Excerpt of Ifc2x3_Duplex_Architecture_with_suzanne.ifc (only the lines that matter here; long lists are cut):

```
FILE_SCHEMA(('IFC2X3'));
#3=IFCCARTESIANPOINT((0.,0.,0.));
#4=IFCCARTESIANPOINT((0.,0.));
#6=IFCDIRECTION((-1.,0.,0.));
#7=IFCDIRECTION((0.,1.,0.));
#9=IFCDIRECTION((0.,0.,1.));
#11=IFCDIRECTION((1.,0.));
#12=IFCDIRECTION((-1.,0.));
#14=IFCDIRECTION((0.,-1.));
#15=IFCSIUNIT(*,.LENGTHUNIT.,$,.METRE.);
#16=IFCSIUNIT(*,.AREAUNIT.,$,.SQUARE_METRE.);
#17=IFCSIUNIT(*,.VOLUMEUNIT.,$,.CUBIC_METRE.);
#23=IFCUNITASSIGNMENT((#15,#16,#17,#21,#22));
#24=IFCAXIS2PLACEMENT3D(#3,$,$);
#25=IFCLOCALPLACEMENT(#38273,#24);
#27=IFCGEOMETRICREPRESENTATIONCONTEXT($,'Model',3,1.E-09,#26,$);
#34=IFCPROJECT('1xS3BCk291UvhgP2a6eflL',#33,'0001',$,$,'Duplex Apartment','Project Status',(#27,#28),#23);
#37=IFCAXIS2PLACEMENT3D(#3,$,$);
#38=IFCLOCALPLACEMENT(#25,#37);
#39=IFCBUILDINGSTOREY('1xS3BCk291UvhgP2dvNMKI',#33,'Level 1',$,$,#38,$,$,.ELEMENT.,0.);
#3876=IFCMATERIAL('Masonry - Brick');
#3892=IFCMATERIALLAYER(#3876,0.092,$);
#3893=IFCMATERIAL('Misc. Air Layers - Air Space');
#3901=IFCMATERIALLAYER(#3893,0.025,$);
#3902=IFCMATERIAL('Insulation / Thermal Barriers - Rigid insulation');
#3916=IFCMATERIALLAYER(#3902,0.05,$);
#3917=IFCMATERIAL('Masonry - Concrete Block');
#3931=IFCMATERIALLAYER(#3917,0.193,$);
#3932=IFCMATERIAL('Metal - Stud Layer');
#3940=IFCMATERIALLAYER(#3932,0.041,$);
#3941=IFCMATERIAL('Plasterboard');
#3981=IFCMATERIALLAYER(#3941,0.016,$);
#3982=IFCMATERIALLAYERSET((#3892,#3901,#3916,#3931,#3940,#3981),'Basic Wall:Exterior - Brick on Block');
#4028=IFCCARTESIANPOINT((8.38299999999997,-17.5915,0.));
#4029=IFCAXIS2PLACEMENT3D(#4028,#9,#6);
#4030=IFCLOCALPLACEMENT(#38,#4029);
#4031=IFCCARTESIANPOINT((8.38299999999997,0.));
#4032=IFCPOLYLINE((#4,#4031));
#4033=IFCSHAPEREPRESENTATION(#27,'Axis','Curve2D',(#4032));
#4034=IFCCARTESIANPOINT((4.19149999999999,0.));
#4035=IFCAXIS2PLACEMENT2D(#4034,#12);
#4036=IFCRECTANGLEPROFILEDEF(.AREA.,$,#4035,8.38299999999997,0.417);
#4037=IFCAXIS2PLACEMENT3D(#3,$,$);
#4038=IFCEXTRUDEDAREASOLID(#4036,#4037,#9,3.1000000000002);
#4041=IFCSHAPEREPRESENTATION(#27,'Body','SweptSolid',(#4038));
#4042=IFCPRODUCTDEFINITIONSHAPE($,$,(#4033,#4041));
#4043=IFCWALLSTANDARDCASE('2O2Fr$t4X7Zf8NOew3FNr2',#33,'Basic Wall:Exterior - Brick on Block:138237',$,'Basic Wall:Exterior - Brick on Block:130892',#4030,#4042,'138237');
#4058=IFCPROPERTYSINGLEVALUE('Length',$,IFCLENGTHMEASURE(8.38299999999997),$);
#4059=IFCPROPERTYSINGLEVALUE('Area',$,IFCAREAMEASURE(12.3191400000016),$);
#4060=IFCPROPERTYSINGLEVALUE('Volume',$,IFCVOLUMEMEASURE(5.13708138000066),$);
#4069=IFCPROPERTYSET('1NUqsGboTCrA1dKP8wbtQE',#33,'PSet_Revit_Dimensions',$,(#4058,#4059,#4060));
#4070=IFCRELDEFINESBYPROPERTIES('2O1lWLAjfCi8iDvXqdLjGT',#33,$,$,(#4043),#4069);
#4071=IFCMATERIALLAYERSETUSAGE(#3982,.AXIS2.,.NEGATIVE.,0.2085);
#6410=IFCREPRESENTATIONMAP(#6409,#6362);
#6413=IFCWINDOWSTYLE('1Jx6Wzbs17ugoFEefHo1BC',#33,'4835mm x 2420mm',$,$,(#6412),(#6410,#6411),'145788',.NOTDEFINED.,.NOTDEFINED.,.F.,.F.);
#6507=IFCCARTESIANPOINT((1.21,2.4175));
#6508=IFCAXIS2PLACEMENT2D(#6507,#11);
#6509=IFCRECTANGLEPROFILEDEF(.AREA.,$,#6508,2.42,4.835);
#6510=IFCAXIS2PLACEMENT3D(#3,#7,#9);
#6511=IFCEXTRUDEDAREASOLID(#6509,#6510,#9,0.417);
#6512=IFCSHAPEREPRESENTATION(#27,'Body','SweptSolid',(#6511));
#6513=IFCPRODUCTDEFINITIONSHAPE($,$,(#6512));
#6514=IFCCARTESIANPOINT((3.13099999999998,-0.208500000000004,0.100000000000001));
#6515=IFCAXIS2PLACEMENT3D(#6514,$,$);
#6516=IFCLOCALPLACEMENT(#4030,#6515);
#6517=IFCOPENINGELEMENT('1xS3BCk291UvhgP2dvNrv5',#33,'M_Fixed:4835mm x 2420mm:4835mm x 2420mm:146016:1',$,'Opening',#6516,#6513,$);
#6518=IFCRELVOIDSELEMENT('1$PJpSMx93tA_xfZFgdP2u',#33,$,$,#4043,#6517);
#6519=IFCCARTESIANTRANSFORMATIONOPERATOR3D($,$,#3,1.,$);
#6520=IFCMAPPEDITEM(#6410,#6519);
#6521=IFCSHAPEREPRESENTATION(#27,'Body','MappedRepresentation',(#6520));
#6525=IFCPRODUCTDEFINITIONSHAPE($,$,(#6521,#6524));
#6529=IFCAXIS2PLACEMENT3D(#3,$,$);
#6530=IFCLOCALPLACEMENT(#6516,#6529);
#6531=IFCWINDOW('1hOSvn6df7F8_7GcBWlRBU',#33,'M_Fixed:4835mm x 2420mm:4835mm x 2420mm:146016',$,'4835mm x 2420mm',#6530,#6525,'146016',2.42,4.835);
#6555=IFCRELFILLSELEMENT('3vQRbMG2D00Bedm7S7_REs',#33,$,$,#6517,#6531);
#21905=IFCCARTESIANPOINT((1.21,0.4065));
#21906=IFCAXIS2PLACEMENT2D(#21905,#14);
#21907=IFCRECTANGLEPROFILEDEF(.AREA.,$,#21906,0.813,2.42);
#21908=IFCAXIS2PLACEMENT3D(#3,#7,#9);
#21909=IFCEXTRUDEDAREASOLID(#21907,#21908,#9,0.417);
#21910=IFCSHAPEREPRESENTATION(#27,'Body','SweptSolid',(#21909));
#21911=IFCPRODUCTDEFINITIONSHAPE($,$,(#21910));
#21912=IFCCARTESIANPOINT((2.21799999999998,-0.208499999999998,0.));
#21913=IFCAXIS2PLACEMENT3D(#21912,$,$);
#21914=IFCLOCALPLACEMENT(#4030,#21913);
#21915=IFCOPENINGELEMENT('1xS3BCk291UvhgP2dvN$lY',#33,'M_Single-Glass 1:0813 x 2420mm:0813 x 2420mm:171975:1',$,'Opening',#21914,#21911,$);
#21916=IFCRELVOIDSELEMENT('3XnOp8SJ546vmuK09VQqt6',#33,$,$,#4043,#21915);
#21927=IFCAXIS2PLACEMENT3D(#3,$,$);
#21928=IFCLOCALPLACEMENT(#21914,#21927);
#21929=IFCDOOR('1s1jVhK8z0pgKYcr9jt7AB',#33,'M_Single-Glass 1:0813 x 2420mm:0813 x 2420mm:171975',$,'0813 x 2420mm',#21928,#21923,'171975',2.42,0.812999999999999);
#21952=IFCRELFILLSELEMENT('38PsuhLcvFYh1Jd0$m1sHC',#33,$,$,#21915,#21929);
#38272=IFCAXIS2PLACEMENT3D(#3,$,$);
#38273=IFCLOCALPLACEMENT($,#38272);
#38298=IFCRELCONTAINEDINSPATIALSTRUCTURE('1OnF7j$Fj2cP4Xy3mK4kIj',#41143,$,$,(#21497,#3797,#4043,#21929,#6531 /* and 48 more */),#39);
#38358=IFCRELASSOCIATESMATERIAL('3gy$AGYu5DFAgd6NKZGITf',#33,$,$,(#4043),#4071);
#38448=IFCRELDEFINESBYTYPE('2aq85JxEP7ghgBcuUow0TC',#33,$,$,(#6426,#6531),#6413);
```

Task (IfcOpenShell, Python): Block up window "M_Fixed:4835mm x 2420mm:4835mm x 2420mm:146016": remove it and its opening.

```python
import ifcopenshell
import ifcopenshell.api.feature
import ifcopenshell.api.pset
import ifcopenshell.api.root
import ifcopenshell.geom
import ifcopenshell.util.element
import ifcopenshell.util.shape
import ifcopenshell.util.unit

model = ifcopenshell.open("Ifc2x3_Duplex_Architecture_with_suzanne.ifc")
area_scale = ifcopenshell.util.unit.calculate_unit_scale(model, "AREAUNIT")
volume_scale = ifcopenshell.util.unit.calculate_unit_scale(model, "VOLUMEUNIT")
settings = ifcopenshell.geom.settings()


def volume(element):
    """Net volume in cubic metres, openings subtracted."""
    shape = ifcopenshell.geom.create_shape(settings, element)
    return ifcopenshell.util.shape.get_volume(shape.geometry)


window = model.by_guid("1hOSvn6df7F8_7GcBWlRBU")
opening = window.FillsVoids[0].RelatingOpeningElement
wall = opening.VoidsElements[0].RelatingBuildingElement
before = volume(wall)

ifcopenshell.api.root.remove_product(model, product=window)
ifcopenshell.api.feature.remove_feature(model, feature=opening)

after = volume(wall)
thickness = 0.417  # wall thickness in metres

# Update the wall's stored quantities.
pset = model.by_id(ifcopenshell.util.element.get_pset(wall, "PSet_Revit_Dimensions", should_inherit=False)["id"])
ifcopenshell.api.pset.edit_pset(model, pset=pset, properties={
    "Area": model.create_entity("IfcAreaMeasure", after / thickness / area_scale),
    "Volume": model.create_entity("IfcVolumeMeasure", after / volume_scale),
})

print(f"wall volume {before:.3f} -> {after:.3f} m3")

model.write("Ifc2x3_Duplex_Architecture_with_suzanne_v2.ifc")
```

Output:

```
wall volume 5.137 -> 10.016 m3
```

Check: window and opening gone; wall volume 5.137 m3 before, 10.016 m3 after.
